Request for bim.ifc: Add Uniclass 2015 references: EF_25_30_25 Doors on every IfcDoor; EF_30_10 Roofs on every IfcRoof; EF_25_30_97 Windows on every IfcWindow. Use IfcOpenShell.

First a look at what the model holds.

```python
import ifcopenshell

model = ifcopenshell.open("bim.ifc")
print(model.schema)
print("classifications:", [c.Name for c in model.by_type("IfcClassification")])
for ifc_class in ("IfcDoor", "IfcRoof", "IfcStair", "IfcWall", "IfcWindow"):
    print(ifc_class, len(model.by_type(ifc_class)))
```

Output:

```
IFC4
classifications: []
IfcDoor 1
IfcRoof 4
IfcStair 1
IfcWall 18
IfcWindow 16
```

```python
import ifcopenshell
import ifcopenshell.api.classification

model = ifcopenshell.open("bim.ifc")

system = ifcopenshell.api.classification.add_classification(model, classification="Uniclass 2015")

codes = {
    "IfcDoor": ("EF_25_30_25", "Doors"),
    "IfcRoof": ("EF_30_10", "Roofs"),
    "IfcWindow": ("EF_25_30_97", "Windows"),
}
for ifc_class, (code, name) in codes.items():
    products = model.by_type(ifc_class)
    ifcopenshell.api.classification.add_reference(
        model, products=products, classification=system, identification=code, name=name
    )
    print(code, len(products))

model.write("bim_v2.ifc")
```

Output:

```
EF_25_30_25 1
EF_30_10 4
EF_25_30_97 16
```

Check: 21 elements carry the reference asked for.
